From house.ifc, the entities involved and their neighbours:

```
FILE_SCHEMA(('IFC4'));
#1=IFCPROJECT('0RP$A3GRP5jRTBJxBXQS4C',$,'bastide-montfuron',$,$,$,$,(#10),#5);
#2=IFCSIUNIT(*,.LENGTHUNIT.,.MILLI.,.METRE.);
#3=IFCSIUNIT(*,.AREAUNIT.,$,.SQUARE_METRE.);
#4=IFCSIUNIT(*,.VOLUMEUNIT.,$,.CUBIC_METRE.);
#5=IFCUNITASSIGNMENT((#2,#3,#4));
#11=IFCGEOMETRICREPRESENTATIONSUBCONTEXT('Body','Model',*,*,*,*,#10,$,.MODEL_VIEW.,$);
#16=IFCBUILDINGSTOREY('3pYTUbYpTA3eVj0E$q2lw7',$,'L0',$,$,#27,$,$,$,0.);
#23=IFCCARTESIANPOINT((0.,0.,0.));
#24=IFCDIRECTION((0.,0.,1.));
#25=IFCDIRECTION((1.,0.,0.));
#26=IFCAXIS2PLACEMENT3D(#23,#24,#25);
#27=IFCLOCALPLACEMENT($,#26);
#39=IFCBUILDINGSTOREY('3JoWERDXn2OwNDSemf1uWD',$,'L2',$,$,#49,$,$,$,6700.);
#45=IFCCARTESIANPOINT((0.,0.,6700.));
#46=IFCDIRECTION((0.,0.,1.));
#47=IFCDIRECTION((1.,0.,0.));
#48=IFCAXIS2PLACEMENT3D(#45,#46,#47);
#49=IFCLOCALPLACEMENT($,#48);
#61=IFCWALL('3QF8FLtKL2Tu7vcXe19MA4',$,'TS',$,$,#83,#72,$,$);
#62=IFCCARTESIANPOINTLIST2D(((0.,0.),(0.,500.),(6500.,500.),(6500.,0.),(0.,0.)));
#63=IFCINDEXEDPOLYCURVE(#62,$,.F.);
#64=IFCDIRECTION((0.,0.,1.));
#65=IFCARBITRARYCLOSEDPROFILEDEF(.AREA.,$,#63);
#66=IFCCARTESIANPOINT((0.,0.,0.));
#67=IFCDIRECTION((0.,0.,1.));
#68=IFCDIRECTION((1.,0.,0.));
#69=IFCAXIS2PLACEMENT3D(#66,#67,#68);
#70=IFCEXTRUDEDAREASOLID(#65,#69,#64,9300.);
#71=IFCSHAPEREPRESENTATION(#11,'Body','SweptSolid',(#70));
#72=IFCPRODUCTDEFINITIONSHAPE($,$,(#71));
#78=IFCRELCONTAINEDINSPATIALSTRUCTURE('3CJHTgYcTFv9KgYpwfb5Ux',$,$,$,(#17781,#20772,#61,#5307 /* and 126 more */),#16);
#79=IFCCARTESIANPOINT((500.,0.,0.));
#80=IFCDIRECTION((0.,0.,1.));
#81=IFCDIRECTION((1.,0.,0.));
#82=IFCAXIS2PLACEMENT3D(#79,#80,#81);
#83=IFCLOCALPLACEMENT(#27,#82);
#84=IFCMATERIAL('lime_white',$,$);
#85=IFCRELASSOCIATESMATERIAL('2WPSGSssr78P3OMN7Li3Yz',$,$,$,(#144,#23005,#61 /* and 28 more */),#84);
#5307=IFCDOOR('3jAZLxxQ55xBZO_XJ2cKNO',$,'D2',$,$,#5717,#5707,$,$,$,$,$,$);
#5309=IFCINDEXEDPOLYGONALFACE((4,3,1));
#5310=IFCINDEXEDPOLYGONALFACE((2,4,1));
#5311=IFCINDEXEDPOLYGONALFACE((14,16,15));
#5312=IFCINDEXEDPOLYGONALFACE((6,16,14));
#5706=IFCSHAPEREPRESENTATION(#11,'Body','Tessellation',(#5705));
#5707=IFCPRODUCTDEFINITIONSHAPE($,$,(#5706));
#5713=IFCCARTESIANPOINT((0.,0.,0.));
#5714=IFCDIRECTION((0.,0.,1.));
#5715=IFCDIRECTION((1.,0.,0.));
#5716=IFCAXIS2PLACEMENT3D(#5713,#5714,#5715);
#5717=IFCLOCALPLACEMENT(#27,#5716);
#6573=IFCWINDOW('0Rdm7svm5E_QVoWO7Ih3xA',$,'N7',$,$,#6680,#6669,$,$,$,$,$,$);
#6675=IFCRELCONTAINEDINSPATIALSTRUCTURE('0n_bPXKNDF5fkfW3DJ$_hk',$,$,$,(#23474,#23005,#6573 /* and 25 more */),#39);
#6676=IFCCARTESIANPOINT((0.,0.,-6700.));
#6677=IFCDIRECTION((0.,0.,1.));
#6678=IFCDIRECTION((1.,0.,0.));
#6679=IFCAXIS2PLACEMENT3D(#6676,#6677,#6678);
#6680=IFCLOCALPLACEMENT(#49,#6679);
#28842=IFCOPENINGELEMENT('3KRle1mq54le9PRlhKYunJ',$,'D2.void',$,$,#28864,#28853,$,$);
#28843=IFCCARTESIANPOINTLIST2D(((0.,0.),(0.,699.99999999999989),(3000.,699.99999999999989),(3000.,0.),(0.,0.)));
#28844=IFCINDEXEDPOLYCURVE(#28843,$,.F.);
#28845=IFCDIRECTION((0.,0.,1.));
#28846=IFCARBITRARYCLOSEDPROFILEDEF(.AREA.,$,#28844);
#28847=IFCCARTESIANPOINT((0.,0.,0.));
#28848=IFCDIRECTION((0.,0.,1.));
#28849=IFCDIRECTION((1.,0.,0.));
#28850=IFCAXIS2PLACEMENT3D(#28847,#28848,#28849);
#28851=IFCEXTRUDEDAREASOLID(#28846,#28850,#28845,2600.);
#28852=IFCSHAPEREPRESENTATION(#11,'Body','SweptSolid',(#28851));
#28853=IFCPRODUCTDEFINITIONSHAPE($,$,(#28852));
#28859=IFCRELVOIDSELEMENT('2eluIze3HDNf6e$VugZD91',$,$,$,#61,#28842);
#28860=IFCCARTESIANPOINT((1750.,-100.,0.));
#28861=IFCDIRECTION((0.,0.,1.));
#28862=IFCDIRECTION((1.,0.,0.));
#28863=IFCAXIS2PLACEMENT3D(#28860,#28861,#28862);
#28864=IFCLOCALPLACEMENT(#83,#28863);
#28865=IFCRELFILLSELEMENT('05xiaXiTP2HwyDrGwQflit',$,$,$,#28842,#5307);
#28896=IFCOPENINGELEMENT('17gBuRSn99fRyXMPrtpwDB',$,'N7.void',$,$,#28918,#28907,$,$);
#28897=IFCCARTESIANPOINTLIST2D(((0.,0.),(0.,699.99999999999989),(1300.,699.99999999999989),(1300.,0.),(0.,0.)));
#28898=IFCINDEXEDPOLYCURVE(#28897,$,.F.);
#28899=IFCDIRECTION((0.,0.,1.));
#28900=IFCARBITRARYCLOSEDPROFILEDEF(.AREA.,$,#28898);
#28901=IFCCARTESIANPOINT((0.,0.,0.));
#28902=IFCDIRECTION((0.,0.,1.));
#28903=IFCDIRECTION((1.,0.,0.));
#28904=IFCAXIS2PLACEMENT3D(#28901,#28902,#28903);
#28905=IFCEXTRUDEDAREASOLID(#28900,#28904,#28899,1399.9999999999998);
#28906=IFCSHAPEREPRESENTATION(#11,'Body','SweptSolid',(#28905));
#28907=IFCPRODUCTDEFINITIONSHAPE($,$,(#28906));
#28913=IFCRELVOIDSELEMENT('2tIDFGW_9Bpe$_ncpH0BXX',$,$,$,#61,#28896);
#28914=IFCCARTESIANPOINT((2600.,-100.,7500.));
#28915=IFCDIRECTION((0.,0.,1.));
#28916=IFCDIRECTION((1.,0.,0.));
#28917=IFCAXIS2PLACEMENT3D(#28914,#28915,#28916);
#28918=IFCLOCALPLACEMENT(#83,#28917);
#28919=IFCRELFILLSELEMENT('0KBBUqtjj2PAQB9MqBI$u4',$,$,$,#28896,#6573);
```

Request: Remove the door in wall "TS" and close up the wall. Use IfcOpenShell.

```python
import ifcopenshell
import ifcopenshell.api.feature
import ifcopenshell.api.root
import ifcopenshell.geom
import ifcopenshell.util.shape

model = ifcopenshell.open("house.ifc")
settings = ifcopenshell.geom.settings()


def volume(element):
    """Net volume in cubic metres, openings subtracted."""
    shape = ifcopenshell.geom.create_shape(settings, element)
    return ifcopenshell.util.shape.get_volume(shape.geometry)


door = model.by_guid("3jAZLxxQ55xBZO_XJ2cKNO")
opening = door.FillsVoids[0].RelatingOpeningElement
wall = opening.VoidsElements[0].RelatingBuildingElement
before = volume(wall)

ifcopenshell.api.root.remove_product(model, product=door)
ifcopenshell.api.feature.remove_feature(model, feature=opening)

after = volume(wall)

print(f"wall volume {before:.3f} -> {after:.3f} m3")

model.write("house_v2.ifc")
```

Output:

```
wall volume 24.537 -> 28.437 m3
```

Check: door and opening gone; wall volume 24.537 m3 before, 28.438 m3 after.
